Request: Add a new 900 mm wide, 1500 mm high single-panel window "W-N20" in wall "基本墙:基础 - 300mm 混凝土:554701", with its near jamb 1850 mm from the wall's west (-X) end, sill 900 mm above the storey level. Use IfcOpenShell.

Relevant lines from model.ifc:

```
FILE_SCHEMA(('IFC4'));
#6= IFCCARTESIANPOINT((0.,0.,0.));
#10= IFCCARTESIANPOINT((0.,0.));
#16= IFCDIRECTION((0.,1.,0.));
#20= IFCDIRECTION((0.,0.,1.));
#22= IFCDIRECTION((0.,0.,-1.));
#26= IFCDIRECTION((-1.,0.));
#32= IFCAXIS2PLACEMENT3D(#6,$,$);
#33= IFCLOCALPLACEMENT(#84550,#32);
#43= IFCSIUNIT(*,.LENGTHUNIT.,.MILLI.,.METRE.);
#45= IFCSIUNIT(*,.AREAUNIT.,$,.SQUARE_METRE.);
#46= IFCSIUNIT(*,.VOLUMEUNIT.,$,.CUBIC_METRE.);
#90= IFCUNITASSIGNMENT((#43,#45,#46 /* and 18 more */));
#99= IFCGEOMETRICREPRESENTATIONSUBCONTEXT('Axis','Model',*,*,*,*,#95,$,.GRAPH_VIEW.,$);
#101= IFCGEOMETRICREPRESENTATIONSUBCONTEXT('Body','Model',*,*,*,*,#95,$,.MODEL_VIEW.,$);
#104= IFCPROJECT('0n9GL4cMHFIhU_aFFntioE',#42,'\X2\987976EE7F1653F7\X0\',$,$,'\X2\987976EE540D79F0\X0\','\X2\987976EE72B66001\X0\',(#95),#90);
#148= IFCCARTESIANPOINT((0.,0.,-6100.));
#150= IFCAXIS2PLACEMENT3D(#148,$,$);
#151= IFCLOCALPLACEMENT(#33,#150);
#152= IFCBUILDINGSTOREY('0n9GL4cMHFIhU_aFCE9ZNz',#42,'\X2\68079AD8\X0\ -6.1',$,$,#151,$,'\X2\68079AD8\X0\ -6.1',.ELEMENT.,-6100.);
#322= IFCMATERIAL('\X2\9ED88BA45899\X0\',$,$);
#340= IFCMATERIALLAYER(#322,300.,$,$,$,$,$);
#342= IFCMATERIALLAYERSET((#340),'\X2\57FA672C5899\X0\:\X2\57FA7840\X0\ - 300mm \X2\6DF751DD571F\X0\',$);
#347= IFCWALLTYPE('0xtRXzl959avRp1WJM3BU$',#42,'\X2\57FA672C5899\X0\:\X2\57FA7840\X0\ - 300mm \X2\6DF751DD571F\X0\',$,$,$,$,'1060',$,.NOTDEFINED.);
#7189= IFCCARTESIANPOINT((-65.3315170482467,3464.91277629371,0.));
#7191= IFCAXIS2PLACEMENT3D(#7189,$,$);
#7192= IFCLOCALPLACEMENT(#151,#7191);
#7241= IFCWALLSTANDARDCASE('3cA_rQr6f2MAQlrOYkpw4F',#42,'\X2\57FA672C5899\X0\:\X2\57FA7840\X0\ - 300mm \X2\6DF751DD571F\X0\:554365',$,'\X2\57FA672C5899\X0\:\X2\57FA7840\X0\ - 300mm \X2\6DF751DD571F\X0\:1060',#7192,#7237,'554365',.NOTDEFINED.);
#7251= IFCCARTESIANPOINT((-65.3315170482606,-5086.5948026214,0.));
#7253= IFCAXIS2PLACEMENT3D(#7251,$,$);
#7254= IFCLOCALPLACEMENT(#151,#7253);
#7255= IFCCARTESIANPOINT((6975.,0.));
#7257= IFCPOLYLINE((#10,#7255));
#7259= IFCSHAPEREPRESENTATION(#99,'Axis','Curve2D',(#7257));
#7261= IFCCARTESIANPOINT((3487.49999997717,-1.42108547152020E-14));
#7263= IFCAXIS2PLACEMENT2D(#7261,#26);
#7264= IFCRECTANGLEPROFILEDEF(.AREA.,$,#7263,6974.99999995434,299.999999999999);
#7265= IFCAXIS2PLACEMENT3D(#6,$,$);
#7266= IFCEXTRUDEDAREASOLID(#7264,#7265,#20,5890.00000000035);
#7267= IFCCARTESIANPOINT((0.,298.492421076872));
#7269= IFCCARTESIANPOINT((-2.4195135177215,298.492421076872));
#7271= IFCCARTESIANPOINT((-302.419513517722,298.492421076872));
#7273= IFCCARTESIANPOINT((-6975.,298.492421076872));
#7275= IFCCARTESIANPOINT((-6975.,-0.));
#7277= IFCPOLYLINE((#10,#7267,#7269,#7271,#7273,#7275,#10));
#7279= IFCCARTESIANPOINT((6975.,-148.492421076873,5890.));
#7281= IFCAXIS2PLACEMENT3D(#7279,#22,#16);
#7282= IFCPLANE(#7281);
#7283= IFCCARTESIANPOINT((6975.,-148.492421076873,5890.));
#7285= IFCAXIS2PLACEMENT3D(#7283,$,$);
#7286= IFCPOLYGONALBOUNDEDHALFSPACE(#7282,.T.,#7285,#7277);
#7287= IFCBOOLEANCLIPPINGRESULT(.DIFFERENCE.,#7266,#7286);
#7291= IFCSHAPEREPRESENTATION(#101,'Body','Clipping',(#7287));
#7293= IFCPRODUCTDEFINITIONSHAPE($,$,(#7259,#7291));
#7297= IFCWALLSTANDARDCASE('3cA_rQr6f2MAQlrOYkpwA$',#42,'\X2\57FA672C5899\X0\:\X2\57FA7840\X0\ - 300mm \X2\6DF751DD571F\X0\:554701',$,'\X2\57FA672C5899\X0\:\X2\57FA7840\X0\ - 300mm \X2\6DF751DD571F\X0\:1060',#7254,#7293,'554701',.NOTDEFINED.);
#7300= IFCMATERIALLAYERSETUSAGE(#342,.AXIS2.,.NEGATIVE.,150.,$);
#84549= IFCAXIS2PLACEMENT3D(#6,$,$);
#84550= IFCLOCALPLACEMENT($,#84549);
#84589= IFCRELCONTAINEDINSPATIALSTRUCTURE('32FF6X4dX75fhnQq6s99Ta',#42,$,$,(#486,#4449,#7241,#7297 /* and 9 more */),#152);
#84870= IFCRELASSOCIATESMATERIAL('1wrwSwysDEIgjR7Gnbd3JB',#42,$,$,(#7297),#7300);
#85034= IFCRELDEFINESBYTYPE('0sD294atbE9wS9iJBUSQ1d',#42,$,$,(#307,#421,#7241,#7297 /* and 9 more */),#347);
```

```python
import numpy as np
import ifcopenshell
import ifcopenshell.api.feature
import ifcopenshell.api.geometry
import ifcopenshell.api.root
import ifcopenshell.api.spatial
import ifcopenshell.geom
import ifcopenshell.util.element
import ifcopenshell.util.placement
import ifcopenshell.util.representation
import ifcopenshell.util.shape
import ifcopenshell.util.unit

model = ifcopenshell.open("model.ifc")
unit_scale = ifcopenshell.util.unit.calculate_unit_scale(model)
settings = ifcopenshell.geom.settings()


def volume(element):
    """Net volume in cubic metres, openings subtracted."""
    shape = ifcopenshell.geom.create_shape(settings, element)
    return ifcopenshell.util.shape.get_volume(shape.geometry)


wall = model.by_guid("3cA_rQr6f2MAQlrOYkpwA$")
storey = ifcopenshell.util.element.get_container(wall, ifc_class="IfcBuildingStorey")
context = ifcopenshell.util.representation.get_context(model, "Model", "Body", "MODEL_VIEW")
before = volume(wall)

width, height, from_end, sill = 0.9, 1.5, 1.85, 0.9  # metres

# The wall runs along its own X axis, and the end named is its -X end.
wall_shape = ifcopenshell.geom.create_shape(settings, wall)
x, y, z = ifcopenshell.util.shape.get_vertices(wall_shape.geometry).T
start = x.min() + from_end
face, thickness = float(y.min()), float(y.max() - y.min())
wall_matrix = ifcopenshell.util.placement.get_local_placement(wall.ObjectPlacement)
level = ifcopenshell.util.placement.get_local_placement(storey.ObjectPlacement)[2, 3]


def in_wall(x, y):
    """Placement at x, y metres in the wall's axes, at sill height."""
    matrix = wall_matrix.copy()
    matrix[:, 3] = wall_matrix @ np.array([x / unit_scale, y / unit_scale, 0.0, 1.0])
    matrix[2, 3] = level + sill / unit_scale
    return matrix


# Opening: a box that overshoots both wall faces by 50 mm.
opening = ifcopenshell.api.root.create_entity(model, ifc_class="IfcOpeningElement", predefined_type="OPENING")
box = ifcopenshell.api.geometry.add_wall_representation(
    model, context=context, length=width, height=height, thickness=thickness + 0.1
)
ifcopenshell.api.geometry.assign_representation(model, product=opening, representation=box)
ifcopenshell.api.geometry.edit_object_placement(model, product=opening, matrix=in_wall(start, face - 0.05), is_si=False)
ifcopenshell.api.feature.add_feature(model, feature=opening, element=wall)

window = ifcopenshell.api.root.create_entity(model, ifc_class="IfcWindow", name="W-N20", predefined_type="WINDOW")
window.OverallWidth, window.OverallHeight = width / unit_scale, height / unit_scale
window.PartitioningType = "SINGLE_PANEL"
body = ifcopenshell.api.geometry.add_window_representation(
    model,
    context=context,
    overall_width=window.OverallWidth,
    overall_height=window.OverallHeight,
    partition_type="SINGLE_PANEL",
)
ifcopenshell.api.geometry.assign_representation(model, product=window, representation=body)
ifcopenshell.api.spatial.assign_container(model, products=[window], relating_structure=storey)
ifcopenshell.api.feature.add_filling(model, opening=opening, element=window)

# Centre the window in the wall's thickness.
ifcopenshell.api.geometry.edit_object_placement(model, product=window, matrix=in_wall(start, face), is_si=False)
window_shape = ifcopenshell.geom.create_shape(settings, window)
depth = ifcopenshell.util.shape.get_vertices(window_shape.geometry)[:, 1]
offset = face + thickness / 2 - (depth.min() + depth.max()) / 2
ifcopenshell.api.geometry.edit_object_placement(model, product=window, matrix=in_wall(start, offset), is_si=False)

after = volume(wall)

print(f"wall volume {before:.3f} -> {after:.3f} m3")

model.write("model_updated.ifc")
```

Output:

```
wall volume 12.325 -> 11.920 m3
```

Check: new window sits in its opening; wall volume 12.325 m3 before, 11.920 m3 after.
